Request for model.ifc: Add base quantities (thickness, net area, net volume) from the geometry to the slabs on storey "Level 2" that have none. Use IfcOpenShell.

First a look at what the model holds.

```python
import ifcopenshell
import ifcopenshell.util.element
import ifcopenshell.util.unit

model = ifcopenshell.open("model.ifc")
print(model.schema)
for unit_type in ("LENGTHUNIT", "AREAUNIT", "VOLUMEUNIT"):
    print(unit_type, ifcopenshell.util.unit.calculate_unit_scale(model, unit_type))
storey = next(s for s in model.by_type("IfcBuildingStorey") if s.Name == "Level 2")
slabs = [e for e in ifcopenshell.util.element.get_decomposition(storey) if e.is_a("IfcSlab")]
for e in sorted(slabs, key=lambda e: e.id()):
    print(e.id(), e.is_a(), e.Name, list(ifcopenshell.util.element.get_psets(e, qtos_only=True)), sep=" | ")
```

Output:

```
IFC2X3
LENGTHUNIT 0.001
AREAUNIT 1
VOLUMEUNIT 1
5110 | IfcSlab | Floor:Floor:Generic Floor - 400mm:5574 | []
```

```python
import ifcopenshell
import ifcopenshell.api.pset
import ifcopenshell.geom
import ifcopenshell.util.element
import ifcopenshell.util.shape
import ifcopenshell.util.unit

model = ifcopenshell.open("model.ifc")
unit_scale = ifcopenshell.util.unit.calculate_unit_scale(model)
area_scale = ifcopenshell.util.unit.calculate_unit_scale(model, "AREAUNIT")
volume_scale = ifcopenshell.util.unit.calculate_unit_scale(model, "VOLUMEUNIT")
settings = ifcopenshell.geom.settings()

storey = next(s for s in model.by_type("IfcBuildingStorey") if s.Name == "Level 2")
slabs = [e for e in ifcopenshell.util.element.get_decomposition(storey) if e.is_a("IfcSlab")]

for e in sorted(slabs, key=lambda e: e.id()):
    if ifcopenshell.util.element.get_psets(e, qtos_only=True, should_inherit=False):
        continue
    # Geometry comes back in metres, in the element's own axes.
    shape = ifcopenshell.geom.create_shape(settings, e)
    values = {
        "Width": ifcopenshell.util.shape.get_z(shape.geometry) / unit_scale,
        "NetArea": ifcopenshell.util.shape.get_footprint_area(shape.geometry) / area_scale,
        "NetVolume": ifcopenshell.util.shape.get_volume(shape.geometry) / volume_scale,
    }
    qto = ifcopenshell.api.pset.add_qto(model, product=e, name="BaseQuantities")
    ifcopenshell.api.pset.edit_qto(model, qto=qto, properties=values)
    print(e.id(), {k: round(v, 3) for k, v in values.items()})

model.write("model-out.ifc")
```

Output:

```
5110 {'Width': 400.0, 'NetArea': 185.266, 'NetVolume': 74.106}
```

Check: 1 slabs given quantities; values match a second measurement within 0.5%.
